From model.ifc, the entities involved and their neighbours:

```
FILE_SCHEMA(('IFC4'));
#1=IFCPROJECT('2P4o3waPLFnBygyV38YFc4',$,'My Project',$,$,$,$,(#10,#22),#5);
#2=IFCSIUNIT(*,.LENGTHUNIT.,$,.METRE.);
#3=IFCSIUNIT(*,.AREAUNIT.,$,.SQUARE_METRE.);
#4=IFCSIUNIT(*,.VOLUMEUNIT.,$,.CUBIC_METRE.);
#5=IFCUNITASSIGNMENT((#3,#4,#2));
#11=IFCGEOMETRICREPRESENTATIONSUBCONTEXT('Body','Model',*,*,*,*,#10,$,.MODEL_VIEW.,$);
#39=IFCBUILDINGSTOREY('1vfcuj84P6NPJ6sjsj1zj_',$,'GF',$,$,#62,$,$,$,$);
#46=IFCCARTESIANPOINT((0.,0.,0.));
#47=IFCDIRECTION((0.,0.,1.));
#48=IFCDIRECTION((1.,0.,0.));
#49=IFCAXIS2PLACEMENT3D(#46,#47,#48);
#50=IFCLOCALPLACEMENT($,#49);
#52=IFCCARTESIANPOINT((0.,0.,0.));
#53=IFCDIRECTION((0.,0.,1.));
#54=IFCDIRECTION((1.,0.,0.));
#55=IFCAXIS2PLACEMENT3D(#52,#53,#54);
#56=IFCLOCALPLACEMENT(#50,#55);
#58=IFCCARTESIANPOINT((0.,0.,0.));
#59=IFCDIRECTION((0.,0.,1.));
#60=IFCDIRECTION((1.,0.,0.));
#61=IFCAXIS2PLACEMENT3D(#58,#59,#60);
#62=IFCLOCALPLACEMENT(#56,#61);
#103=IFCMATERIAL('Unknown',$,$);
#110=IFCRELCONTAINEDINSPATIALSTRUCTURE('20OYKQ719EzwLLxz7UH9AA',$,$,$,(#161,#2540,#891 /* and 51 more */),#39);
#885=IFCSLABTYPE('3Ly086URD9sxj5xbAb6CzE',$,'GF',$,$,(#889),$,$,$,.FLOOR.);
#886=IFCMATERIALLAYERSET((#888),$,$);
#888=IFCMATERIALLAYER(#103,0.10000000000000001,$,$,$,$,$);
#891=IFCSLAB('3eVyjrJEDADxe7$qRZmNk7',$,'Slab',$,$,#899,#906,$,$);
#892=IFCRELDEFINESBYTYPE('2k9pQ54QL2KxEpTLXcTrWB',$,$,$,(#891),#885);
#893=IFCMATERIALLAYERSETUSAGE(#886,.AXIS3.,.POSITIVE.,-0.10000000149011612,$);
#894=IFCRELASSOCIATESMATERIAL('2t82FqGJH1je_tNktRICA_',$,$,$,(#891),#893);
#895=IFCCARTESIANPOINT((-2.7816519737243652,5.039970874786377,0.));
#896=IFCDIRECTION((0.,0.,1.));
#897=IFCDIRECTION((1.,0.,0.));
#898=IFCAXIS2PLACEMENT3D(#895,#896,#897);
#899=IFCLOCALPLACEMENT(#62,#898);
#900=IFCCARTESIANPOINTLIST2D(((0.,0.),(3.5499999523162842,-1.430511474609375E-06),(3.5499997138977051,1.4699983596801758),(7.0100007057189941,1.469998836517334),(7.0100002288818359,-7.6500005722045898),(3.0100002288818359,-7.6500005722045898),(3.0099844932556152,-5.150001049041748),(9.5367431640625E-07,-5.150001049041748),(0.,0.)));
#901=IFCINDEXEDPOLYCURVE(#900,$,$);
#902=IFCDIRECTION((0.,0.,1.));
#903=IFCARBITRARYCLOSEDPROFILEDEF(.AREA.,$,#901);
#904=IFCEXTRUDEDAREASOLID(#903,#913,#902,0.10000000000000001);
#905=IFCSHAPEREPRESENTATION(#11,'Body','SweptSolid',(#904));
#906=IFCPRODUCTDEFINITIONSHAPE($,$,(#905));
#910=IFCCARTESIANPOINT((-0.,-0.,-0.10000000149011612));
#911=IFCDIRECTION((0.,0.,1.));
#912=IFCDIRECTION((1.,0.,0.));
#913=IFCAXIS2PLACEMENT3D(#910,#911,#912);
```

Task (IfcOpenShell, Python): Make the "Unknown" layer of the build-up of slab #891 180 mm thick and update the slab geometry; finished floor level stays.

```python
import ifcopenshell
import ifcopenshell.util.element
import ifcopenshell.util.representation

model = ifcopenshell.open("model.ifc")

layer_set = model.by_id(886)
layer = next(l for l in layer_set.MaterialLayers if l.Material and l.Material.Name == "Unknown")
change = 0.18 - layer.LayerThickness
layer.LayerThickness += change

# Geometry does not follow the layer set by itself.
slabs = [e for e in ifcopenshell.util.element.get_elements_by_material(model, layer_set) if e.is_a("IfcSlab")]
for slab in sorted(slabs, key=lambda e: e.id()):
    body = ifcopenshell.util.representation.get_representation(slab, "Model", "Body")
    solid = body.Items[0]
    old_depth = solid.Depth
    solid.Depth += change
    # Extruded upwards: lower the start of the extrusion so the top stays.
    x, y, z = solid.Position.Location.Coordinates
    solid.Position.Location = model.createIfcCartesianPoint((x, y, z - change))
    print(slab.id(), f"{old_depth:g} -> {solid.Depth:g}")

# The layers are counted up from the underside, which has moved.
for usage in {ifcopenshell.util.element.get_material(slab) for slab in slabs}:
    usage.OffsetFromReferenceLine -= change

model.write("model_v2.ifc")
```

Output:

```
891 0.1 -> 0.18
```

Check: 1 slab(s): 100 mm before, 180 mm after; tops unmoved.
